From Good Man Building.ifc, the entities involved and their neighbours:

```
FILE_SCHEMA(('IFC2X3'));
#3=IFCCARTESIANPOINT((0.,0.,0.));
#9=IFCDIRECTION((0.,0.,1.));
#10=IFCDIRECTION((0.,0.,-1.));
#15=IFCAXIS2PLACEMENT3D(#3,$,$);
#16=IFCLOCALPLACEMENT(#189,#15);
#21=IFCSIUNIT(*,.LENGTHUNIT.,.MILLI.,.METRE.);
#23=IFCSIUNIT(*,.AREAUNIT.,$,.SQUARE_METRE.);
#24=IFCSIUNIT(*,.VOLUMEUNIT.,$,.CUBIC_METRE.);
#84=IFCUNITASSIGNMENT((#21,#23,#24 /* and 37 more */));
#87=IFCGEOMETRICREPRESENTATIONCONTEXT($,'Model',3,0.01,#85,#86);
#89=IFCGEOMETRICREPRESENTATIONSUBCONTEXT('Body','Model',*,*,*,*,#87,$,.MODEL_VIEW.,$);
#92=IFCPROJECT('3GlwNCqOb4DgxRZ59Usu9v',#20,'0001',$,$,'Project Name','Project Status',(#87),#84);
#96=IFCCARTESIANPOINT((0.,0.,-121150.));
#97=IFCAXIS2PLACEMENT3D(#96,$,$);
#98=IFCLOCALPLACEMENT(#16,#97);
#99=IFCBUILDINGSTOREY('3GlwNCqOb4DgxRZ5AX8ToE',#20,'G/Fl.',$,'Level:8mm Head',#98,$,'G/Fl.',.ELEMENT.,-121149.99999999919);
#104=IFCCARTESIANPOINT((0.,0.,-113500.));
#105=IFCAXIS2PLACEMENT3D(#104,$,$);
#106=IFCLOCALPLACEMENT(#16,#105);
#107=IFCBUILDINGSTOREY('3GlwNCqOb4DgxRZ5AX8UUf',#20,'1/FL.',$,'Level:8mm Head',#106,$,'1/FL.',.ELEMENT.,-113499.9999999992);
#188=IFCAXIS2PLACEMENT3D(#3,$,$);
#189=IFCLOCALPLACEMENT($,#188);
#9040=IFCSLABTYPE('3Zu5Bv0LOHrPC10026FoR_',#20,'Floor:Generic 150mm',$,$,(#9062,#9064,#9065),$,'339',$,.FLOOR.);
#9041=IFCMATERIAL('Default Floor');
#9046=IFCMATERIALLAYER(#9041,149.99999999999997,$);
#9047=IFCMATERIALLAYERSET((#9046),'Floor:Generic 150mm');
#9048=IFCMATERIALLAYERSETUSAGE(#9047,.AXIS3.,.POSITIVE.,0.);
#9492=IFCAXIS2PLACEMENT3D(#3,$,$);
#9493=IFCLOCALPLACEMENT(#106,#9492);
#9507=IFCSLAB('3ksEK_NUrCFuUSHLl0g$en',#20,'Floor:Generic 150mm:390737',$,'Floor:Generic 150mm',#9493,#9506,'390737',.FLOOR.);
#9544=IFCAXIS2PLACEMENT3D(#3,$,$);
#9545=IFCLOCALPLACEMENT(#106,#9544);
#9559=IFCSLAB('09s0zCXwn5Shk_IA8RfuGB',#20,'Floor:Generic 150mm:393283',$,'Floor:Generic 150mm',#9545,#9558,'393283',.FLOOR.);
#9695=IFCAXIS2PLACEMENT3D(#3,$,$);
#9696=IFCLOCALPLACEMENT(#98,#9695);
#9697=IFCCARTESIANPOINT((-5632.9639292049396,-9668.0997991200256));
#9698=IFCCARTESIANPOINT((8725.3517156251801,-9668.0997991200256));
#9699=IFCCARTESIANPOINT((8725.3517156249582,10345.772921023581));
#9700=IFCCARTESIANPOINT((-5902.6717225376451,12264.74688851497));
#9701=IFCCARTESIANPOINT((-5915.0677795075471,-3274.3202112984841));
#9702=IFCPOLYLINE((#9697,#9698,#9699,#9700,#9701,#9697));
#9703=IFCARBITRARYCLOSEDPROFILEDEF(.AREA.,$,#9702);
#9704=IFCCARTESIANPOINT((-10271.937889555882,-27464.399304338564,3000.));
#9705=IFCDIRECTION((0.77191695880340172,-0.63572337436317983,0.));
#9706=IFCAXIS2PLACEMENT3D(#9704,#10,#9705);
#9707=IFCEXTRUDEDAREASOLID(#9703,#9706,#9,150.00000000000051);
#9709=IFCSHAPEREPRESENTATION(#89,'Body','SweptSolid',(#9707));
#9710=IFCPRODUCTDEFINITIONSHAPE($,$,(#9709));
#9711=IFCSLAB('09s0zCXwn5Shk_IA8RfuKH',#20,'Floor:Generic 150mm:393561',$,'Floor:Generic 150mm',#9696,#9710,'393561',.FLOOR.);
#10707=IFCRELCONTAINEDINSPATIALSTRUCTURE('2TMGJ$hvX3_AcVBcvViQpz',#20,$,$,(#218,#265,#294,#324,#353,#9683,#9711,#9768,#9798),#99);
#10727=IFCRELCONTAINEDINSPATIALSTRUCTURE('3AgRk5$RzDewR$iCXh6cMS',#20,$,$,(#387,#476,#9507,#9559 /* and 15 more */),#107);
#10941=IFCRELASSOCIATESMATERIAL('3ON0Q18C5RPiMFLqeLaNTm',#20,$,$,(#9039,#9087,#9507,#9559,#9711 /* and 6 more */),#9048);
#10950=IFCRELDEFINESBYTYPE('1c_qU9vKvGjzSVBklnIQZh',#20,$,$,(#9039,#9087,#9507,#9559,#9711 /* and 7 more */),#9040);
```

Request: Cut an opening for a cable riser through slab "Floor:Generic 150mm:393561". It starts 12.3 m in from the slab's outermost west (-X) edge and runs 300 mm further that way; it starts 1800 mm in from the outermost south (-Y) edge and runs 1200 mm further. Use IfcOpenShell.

```python
import numpy as np
import ifcopenshell
import ifcopenshell.api.feature
import ifcopenshell.api.geometry
import ifcopenshell.api.root
import ifcopenshell.geom
import ifcopenshell.util.placement
import ifcopenshell.util.representation
import ifcopenshell.util.shape
import ifcopenshell.util.unit

model = ifcopenshell.open("Good Man Building.ifc")
unit_scale = ifcopenshell.util.unit.calculate_unit_scale(model)
settings = ifcopenshell.geom.settings()


def volume(element):
    """Net volume in cubic metres, openings subtracted."""
    shape = ifcopenshell.geom.create_shape(settings, element)
    return ifcopenshell.util.shape.get_volume(shape.geometry)


slab = model.by_id(9711)
before = volume(slab)

# Extent in the slab's own axes, in metres. The edges named are its -X and -Y sides.
slab_shape = ifcopenshell.geom.create_shape(settings, slab)
vertices = ifcopenshell.util.shape.get_vertices(slab_shape.geometry)
x_min, y_min, bottom = vertices.min(axis=0)
top = vertices[:, 2].max()

opening = ifcopenshell.api.root.create_entity(model, ifc_class="IfcOpeningElement", name="Cable riser opening")
context = ifcopenshell.util.representation.get_context(model, "Model", "Body", "MODEL_VIEW")
width, depth = 0.3, 1.2
outline = [(0.0, 0.0), (width, 0.0), (width, depth), (0.0, depth), (0.0, 0.0)]
# Overshoot both faces by 50 mm so the cut is clean.
shape = ifcopenshell.api.geometry.add_slab_representation(
    model, context=context, depth=top - bottom + 0.1, polyline=outline
)
ifcopenshell.api.geometry.assign_representation(model, product=opening, representation=shape)

matrix = ifcopenshell.util.placement.get_local_placement(slab.ObjectPlacement)
matrix[:, 3] = matrix @ np.append(np.array([x_min + 12.3, y_min + 1.8, bottom - 0.05]) / unit_scale, 1.0)
ifcopenshell.api.geometry.edit_object_placement(model, product=opening, matrix=matrix, is_si=False)
ifcopenshell.api.feature.add_feature(model, feature=opening, element=slab)

after = volume(slab)

print(f"slab volume {before:.3f} -> {after:.3f} m3")

model.write("Good Man Building-out.ifc")
```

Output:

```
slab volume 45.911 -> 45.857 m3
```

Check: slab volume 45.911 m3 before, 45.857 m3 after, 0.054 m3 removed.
